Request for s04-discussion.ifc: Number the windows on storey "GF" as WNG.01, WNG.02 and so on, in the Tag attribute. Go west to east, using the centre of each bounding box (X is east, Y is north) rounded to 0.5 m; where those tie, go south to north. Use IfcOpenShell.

First a look at what the model holds.

```python
import ifcopenshell
import ifcopenshell.util.element
import ifcopenshell.util.placement

model = ifcopenshell.open("s04-discussion.ifc")
print(model.schema)
storey = next(s for s in model.by_type("IfcBuildingStorey") if s.Name == "GF")
windows = [e for e in ifcopenshell.util.element.get_decomposition(storey) if e.is_a("IfcWindow")]
for e in sorted(windows, key=lambda e: e.id()):
    origin = ifcopenshell.util.placement.get_local_placement(e.ObjectPlacement)[:3, 3]
    print(e.id(), e.Tag, e.Name, origin.round(2) + 0.0, sep=" | ")
```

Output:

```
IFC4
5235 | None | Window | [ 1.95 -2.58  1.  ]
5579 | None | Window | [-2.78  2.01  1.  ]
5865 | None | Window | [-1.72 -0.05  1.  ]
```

```python
import ifcopenshell
import ifcopenshell.geom
import ifcopenshell.util.element
import ifcopenshell.util.shape

model = ifcopenshell.open("s04-discussion.ifc")
settings = ifcopenshell.geom.settings()
settings.set("use-world-coords", True)


def centre(element):
    shape = ifcopenshell.geom.create_shape(settings, element)
    return ifcopenshell.util.shape.get_bbox_centroid(shape.geometry)


storey = next(s for s in model.by_type("IfcBuildingStorey") if s.Name == "GF")
windows = [e for e in ifcopenshell.util.element.get_decomposition(storey) if e.is_a("IfcWindow")]

# Insertion points can sit at a corner or the storey origin, so sort by the geometry (in metres).
centres = {e: centre(e) for e in windows}
windows.sort(key=lambda e: (round(centres[e][0] / 0.5), centres[e][1]))

for i, e in enumerate(windows, start=1):
    number = f"WNG.{i:02d}"
    e.Tag = number
    print(e.id(), number)

model.write("s04-discussion_v2.ifc")
```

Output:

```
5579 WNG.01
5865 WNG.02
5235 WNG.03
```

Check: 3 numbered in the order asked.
